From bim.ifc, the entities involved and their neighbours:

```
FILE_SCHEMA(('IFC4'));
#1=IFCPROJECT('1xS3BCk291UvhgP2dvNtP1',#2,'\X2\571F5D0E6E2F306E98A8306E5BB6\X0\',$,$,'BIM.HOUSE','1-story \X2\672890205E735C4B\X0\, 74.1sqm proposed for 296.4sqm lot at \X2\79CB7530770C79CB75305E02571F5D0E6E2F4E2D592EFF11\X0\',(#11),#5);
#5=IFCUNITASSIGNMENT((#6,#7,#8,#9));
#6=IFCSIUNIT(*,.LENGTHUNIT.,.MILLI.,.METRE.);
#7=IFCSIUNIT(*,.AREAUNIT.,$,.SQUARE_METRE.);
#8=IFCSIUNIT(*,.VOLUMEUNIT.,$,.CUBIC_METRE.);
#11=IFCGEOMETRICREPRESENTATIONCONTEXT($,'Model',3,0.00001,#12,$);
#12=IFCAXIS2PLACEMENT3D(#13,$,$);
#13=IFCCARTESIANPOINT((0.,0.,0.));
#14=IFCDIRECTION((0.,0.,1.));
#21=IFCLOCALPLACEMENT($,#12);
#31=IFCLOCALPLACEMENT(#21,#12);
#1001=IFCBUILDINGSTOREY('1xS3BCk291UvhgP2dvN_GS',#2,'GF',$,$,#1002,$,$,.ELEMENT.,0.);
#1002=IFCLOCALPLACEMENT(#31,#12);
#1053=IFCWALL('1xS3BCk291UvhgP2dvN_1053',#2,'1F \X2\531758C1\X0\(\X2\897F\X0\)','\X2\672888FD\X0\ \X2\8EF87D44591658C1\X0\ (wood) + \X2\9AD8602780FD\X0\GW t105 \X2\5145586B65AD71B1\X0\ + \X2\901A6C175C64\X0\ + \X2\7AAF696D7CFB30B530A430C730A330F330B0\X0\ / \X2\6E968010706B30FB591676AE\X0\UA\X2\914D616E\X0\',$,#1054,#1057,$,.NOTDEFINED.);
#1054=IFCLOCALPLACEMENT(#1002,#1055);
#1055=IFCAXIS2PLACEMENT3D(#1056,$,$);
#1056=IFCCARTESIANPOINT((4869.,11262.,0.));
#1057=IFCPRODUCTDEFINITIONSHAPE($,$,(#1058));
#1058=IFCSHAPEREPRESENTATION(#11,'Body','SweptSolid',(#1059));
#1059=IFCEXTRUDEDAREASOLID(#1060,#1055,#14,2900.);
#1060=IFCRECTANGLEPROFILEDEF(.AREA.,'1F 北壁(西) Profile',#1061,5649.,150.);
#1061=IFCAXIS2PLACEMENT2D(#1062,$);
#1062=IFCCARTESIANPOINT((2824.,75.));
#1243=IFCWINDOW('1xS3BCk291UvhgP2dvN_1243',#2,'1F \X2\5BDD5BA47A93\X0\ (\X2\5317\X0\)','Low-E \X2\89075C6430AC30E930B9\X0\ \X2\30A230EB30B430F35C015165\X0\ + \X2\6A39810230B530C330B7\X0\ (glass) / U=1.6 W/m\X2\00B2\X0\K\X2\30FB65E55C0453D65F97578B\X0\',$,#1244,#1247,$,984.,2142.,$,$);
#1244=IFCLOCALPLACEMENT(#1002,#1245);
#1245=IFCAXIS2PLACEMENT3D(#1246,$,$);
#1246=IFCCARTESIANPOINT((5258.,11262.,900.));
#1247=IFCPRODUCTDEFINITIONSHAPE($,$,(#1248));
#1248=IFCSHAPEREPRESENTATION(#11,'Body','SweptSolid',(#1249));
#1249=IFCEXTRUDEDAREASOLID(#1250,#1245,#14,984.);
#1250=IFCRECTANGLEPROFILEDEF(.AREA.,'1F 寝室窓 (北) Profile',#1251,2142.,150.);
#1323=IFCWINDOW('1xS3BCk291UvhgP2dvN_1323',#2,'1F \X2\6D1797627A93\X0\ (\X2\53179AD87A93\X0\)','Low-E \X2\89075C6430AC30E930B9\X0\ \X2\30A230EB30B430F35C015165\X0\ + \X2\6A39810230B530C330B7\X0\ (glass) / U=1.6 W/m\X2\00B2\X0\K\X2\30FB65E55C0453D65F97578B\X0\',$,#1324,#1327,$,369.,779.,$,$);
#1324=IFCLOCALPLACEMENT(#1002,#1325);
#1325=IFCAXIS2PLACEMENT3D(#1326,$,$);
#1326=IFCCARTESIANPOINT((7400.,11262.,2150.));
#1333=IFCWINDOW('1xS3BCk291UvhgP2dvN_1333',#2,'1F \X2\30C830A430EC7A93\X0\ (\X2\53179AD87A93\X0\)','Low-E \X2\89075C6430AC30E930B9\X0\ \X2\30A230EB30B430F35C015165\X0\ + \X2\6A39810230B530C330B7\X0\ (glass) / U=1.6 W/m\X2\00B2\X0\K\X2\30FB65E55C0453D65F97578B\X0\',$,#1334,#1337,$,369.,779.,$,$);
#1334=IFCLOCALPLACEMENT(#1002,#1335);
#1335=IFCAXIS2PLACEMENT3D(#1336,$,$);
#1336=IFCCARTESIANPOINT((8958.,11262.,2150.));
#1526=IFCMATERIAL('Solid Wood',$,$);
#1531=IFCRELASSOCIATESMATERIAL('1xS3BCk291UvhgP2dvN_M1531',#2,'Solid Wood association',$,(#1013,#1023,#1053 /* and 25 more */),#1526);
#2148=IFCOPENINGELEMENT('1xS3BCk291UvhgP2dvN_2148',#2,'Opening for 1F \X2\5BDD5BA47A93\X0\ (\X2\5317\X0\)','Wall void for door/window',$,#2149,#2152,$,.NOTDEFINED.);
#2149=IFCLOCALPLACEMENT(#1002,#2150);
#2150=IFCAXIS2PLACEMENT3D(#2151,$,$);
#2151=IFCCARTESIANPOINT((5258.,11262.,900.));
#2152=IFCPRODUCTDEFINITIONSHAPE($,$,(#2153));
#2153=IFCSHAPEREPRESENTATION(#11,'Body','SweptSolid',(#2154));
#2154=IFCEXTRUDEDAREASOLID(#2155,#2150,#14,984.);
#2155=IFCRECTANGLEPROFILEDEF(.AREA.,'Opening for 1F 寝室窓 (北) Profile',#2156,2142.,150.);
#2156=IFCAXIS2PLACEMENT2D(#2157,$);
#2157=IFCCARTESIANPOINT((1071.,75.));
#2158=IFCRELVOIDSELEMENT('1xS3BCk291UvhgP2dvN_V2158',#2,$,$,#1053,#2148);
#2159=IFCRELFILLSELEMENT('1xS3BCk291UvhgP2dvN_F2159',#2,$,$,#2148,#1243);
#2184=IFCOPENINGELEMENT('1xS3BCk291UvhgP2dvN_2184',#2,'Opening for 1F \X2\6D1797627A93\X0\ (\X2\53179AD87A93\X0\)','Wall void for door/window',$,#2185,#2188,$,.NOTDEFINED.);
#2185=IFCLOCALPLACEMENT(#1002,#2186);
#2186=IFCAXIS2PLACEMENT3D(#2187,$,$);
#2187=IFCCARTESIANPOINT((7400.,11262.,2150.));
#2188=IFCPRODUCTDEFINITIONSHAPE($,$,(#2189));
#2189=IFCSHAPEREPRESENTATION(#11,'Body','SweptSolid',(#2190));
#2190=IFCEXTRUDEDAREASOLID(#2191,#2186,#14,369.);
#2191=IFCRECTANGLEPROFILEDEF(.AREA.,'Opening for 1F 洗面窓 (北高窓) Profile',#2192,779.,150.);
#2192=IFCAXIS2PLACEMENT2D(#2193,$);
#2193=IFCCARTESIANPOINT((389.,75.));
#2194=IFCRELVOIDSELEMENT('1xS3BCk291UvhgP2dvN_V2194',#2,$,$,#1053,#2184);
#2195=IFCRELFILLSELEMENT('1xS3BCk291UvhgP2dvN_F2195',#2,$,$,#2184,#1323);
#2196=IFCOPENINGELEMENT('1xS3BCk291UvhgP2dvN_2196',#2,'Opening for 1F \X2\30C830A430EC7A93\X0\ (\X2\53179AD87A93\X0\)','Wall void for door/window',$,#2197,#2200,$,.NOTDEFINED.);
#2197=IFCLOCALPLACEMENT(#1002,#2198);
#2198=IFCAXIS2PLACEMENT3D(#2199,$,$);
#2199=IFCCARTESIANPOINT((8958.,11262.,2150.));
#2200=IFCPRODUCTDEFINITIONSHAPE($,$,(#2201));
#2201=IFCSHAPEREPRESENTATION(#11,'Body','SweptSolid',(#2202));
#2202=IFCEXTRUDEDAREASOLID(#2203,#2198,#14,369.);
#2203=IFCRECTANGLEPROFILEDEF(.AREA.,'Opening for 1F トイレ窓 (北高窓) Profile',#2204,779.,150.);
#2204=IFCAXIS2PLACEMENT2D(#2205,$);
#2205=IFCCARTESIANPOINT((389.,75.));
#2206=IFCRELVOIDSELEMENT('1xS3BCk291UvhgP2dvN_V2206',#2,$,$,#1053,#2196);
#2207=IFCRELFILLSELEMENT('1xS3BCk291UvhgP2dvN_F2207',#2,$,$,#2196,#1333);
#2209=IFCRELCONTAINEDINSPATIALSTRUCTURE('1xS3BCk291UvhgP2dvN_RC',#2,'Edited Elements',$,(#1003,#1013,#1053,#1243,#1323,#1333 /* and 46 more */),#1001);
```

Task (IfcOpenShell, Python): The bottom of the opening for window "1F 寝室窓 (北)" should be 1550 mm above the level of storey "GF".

```python
import numpy as np
import ifcopenshell
import ifcopenshell.api.geometry
import ifcopenshell.geom
import ifcopenshell.util.element
import ifcopenshell.util.placement
import ifcopenshell.util.shape
import ifcopenshell.util.unit

model = ifcopenshell.open("bim.ifc")
unit_scale = ifcopenshell.util.unit.calculate_unit_scale(model)

window = model.by_guid("1xS3BCk291UvhgP2dvN_1243")
opening = window.FillsVoids[0].RelatingOpeningElement
storey = ifcopenshell.util.element.get_container(window, ifc_class="IfcBuildingStorey")
level = ifcopenshell.util.placement.get_local_placement(storey.ObjectPlacement)[2, 3]

# The opening's origin need not be at the sill, so measure its lowest point.
shape = ifcopenshell.geom.create_shape(ifcopenshell.geom.settings(), opening)
bottom = ifcopenshell.util.shape.get_shape_bottom_elevation(shape, shape.geometry) / unit_scale
dz = level + 1550.0 - bottom

shift = np.array([0.0, 0.0, dz])
# The window is not placed relative to its opening, so move both.
for product in (opening, window):
    matrix = ifcopenshell.util.placement.get_local_placement(product.ObjectPlacement)
    matrix[:3, 3] += shift
    ifcopenshell.api.geometry.edit_object_placement(model, product=product, matrix=matrix, is_si=False)

print(f"moved by {dz * unit_scale:+.3f} m")

model.write("bim-out.ifc")
```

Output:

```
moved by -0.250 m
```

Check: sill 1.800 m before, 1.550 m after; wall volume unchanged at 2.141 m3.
